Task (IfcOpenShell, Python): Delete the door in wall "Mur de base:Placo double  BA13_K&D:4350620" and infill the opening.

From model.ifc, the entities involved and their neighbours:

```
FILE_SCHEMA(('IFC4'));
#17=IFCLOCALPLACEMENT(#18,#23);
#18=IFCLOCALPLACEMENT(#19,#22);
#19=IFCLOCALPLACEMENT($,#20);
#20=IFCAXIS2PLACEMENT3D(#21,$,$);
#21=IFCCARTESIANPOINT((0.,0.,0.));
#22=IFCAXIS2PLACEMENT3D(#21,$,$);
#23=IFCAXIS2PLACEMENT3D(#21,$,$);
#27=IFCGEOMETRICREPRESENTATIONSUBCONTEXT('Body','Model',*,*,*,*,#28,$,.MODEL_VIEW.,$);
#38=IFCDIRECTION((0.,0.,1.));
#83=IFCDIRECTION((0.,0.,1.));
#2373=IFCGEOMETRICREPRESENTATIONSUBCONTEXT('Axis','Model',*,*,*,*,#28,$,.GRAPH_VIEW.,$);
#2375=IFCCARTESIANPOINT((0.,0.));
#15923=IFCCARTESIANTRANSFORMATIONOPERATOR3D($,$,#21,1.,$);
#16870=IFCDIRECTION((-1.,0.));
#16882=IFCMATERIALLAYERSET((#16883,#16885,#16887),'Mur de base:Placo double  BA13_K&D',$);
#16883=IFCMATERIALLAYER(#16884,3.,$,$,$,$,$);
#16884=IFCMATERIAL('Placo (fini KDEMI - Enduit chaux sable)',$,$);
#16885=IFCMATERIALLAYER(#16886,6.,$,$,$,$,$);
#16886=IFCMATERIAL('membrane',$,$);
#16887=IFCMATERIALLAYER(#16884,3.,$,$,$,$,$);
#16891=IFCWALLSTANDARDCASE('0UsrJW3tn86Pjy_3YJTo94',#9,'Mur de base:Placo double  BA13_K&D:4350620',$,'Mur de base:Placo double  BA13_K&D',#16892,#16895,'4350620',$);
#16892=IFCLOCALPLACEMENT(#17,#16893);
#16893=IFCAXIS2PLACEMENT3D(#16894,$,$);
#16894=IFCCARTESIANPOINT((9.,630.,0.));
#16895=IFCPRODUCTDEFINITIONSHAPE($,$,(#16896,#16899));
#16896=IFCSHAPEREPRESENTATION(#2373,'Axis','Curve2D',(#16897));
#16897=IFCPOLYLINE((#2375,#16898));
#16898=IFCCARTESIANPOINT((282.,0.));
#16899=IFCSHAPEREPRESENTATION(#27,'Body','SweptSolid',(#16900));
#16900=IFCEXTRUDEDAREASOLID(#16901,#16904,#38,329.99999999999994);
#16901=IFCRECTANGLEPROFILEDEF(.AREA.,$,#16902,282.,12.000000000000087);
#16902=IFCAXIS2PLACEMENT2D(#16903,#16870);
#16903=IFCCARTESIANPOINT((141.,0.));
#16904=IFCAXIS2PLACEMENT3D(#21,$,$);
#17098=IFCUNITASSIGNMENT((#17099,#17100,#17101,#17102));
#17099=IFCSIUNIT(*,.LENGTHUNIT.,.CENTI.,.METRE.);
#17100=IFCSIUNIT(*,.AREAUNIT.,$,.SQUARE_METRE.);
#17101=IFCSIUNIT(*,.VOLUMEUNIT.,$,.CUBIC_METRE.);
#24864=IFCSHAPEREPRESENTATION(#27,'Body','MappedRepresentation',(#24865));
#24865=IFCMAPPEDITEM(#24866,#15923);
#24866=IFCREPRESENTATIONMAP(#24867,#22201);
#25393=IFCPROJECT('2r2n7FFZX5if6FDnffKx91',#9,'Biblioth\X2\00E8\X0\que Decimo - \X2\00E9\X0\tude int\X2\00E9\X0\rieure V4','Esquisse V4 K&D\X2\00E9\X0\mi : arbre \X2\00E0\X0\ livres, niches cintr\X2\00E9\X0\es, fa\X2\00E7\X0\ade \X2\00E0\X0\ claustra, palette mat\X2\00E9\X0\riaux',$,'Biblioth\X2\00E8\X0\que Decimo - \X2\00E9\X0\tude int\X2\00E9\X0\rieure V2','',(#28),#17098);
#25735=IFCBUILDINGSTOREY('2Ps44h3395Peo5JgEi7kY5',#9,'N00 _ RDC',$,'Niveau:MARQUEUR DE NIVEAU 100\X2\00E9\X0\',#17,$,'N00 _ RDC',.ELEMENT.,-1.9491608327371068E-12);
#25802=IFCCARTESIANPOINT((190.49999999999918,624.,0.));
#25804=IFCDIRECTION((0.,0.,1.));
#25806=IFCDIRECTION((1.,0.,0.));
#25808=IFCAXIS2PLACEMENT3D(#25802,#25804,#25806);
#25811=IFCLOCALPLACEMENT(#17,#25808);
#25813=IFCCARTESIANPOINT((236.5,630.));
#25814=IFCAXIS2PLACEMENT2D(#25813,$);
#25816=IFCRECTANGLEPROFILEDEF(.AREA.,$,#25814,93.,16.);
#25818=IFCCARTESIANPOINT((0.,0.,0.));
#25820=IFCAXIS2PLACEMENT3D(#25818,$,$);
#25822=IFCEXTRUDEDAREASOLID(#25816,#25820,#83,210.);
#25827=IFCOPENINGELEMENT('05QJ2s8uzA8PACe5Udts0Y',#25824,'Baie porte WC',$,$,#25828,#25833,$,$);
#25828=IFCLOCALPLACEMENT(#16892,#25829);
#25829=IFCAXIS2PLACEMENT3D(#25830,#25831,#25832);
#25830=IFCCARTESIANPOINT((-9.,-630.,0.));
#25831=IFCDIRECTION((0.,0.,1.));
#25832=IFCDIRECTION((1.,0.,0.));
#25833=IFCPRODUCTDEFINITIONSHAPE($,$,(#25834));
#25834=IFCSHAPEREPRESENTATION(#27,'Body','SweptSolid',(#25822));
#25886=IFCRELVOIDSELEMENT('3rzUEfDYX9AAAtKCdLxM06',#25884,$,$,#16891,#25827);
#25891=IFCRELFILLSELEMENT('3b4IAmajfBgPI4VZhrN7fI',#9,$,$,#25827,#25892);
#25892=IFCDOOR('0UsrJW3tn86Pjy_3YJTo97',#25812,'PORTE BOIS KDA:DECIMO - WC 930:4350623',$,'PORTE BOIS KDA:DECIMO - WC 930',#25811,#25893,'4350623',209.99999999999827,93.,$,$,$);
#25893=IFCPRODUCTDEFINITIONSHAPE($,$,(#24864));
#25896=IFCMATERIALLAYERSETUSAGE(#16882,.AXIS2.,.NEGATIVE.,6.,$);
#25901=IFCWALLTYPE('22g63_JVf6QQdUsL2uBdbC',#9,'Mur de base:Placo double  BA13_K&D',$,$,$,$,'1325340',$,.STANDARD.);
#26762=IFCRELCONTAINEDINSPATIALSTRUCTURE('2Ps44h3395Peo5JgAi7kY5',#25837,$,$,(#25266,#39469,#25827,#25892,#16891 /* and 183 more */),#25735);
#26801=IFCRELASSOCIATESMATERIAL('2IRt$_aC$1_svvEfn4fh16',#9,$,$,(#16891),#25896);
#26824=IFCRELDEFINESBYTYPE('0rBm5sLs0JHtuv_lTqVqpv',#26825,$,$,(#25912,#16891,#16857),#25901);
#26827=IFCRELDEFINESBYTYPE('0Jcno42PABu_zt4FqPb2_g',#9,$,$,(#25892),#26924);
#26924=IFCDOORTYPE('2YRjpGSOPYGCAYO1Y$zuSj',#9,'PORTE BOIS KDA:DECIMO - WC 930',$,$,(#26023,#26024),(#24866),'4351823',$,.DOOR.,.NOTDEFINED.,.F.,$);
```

```python
import ifcopenshell
import ifcopenshell.api.feature
import ifcopenshell.api.root
import ifcopenshell.geom
import ifcopenshell.util.shape

model = ifcopenshell.open("model.ifc")
settings = ifcopenshell.geom.settings()


def volume(element):
    """Net volume in cubic metres, openings subtracted."""
    shape = ifcopenshell.geom.create_shape(settings, element)
    return ifcopenshell.util.shape.get_volume(shape.geometry)


door = model.by_guid("0UsrJW3tn86Pjy_3YJTo97")
opening = door.FillsVoids[0].RelatingOpeningElement
wall = opening.VoidsElements[0].RelatingBuildingElement
before = volume(wall)

ifcopenshell.api.root.remove_product(model, product=door)
ifcopenshell.api.feature.remove_feature(model, feature=opening)

after = volume(wall)

print(f"wall volume {before:.3f} -> {after:.3f} m3")

model.write("model_v2.ifc")
```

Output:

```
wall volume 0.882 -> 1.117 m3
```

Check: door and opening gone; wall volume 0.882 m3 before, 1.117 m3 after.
